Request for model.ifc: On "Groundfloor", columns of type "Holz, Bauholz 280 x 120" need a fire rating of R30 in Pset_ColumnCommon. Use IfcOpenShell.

First a look at what the model holds.

```python
import ifcopenshell
import ifcopenshell.util.element

model = ifcopenshell.open("model.ifc")
print(model.schema)
storey = next(s for s in model.by_type("IfcBuildingStorey") if s.Name == "Groundfloor")
columns = [e for e in ifcopenshell.util.element.get_decomposition(storey) if e.is_a("IfcColumn")]
seen = {}
for e in columns:
    element_type = ifcopenshell.util.element.get_type(e)
    key = (element_type.Name if element_type != e and element_type else None, ifcopenshell.util.element.get_pset(e, "Pset_ColumnCommon", "FireRating"))
    seen[key] = seen.get(key, 0) + 1
for (name, value), count in sorted(seen.items(), key=str):
    print(count, "x", name, "|", value)
```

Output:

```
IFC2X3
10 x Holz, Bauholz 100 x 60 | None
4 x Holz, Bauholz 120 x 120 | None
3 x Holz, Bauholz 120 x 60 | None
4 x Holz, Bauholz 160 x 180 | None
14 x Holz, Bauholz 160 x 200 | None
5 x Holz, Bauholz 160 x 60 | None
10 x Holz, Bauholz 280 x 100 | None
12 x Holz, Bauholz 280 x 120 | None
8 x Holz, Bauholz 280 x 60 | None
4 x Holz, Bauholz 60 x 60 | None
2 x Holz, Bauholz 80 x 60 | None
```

```python
import ifcopenshell
import ifcopenshell.api.pset
import ifcopenshell.util.element

model = ifcopenshell.open("model.ifc")

storey = next(s for s in model.by_type("IfcBuildingStorey") if s.Name == "Groundfloor")
columns = [e for e in ifcopenshell.util.element.get_decomposition(storey) if e.is_a("IfcColumn")]

count = 0
for e in columns:
    element_type = ifcopenshell.util.element.get_type(e)
    if element_type in (None, e) or element_type.Name != "Holz, Bauholz 280 x 120":
        continue
    # add_pset returns the element's existing set when there is one.
    pset = ifcopenshell.api.pset.add_pset(model, product=e, name="Pset_ColumnCommon")
    ifcopenshell.api.pset.edit_pset(model, pset=pset, properties={"FireRating": "R30"})
    count += 1

print(count, "columns updated")

model.write("model_updated.ifc")
```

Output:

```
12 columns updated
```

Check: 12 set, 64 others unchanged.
